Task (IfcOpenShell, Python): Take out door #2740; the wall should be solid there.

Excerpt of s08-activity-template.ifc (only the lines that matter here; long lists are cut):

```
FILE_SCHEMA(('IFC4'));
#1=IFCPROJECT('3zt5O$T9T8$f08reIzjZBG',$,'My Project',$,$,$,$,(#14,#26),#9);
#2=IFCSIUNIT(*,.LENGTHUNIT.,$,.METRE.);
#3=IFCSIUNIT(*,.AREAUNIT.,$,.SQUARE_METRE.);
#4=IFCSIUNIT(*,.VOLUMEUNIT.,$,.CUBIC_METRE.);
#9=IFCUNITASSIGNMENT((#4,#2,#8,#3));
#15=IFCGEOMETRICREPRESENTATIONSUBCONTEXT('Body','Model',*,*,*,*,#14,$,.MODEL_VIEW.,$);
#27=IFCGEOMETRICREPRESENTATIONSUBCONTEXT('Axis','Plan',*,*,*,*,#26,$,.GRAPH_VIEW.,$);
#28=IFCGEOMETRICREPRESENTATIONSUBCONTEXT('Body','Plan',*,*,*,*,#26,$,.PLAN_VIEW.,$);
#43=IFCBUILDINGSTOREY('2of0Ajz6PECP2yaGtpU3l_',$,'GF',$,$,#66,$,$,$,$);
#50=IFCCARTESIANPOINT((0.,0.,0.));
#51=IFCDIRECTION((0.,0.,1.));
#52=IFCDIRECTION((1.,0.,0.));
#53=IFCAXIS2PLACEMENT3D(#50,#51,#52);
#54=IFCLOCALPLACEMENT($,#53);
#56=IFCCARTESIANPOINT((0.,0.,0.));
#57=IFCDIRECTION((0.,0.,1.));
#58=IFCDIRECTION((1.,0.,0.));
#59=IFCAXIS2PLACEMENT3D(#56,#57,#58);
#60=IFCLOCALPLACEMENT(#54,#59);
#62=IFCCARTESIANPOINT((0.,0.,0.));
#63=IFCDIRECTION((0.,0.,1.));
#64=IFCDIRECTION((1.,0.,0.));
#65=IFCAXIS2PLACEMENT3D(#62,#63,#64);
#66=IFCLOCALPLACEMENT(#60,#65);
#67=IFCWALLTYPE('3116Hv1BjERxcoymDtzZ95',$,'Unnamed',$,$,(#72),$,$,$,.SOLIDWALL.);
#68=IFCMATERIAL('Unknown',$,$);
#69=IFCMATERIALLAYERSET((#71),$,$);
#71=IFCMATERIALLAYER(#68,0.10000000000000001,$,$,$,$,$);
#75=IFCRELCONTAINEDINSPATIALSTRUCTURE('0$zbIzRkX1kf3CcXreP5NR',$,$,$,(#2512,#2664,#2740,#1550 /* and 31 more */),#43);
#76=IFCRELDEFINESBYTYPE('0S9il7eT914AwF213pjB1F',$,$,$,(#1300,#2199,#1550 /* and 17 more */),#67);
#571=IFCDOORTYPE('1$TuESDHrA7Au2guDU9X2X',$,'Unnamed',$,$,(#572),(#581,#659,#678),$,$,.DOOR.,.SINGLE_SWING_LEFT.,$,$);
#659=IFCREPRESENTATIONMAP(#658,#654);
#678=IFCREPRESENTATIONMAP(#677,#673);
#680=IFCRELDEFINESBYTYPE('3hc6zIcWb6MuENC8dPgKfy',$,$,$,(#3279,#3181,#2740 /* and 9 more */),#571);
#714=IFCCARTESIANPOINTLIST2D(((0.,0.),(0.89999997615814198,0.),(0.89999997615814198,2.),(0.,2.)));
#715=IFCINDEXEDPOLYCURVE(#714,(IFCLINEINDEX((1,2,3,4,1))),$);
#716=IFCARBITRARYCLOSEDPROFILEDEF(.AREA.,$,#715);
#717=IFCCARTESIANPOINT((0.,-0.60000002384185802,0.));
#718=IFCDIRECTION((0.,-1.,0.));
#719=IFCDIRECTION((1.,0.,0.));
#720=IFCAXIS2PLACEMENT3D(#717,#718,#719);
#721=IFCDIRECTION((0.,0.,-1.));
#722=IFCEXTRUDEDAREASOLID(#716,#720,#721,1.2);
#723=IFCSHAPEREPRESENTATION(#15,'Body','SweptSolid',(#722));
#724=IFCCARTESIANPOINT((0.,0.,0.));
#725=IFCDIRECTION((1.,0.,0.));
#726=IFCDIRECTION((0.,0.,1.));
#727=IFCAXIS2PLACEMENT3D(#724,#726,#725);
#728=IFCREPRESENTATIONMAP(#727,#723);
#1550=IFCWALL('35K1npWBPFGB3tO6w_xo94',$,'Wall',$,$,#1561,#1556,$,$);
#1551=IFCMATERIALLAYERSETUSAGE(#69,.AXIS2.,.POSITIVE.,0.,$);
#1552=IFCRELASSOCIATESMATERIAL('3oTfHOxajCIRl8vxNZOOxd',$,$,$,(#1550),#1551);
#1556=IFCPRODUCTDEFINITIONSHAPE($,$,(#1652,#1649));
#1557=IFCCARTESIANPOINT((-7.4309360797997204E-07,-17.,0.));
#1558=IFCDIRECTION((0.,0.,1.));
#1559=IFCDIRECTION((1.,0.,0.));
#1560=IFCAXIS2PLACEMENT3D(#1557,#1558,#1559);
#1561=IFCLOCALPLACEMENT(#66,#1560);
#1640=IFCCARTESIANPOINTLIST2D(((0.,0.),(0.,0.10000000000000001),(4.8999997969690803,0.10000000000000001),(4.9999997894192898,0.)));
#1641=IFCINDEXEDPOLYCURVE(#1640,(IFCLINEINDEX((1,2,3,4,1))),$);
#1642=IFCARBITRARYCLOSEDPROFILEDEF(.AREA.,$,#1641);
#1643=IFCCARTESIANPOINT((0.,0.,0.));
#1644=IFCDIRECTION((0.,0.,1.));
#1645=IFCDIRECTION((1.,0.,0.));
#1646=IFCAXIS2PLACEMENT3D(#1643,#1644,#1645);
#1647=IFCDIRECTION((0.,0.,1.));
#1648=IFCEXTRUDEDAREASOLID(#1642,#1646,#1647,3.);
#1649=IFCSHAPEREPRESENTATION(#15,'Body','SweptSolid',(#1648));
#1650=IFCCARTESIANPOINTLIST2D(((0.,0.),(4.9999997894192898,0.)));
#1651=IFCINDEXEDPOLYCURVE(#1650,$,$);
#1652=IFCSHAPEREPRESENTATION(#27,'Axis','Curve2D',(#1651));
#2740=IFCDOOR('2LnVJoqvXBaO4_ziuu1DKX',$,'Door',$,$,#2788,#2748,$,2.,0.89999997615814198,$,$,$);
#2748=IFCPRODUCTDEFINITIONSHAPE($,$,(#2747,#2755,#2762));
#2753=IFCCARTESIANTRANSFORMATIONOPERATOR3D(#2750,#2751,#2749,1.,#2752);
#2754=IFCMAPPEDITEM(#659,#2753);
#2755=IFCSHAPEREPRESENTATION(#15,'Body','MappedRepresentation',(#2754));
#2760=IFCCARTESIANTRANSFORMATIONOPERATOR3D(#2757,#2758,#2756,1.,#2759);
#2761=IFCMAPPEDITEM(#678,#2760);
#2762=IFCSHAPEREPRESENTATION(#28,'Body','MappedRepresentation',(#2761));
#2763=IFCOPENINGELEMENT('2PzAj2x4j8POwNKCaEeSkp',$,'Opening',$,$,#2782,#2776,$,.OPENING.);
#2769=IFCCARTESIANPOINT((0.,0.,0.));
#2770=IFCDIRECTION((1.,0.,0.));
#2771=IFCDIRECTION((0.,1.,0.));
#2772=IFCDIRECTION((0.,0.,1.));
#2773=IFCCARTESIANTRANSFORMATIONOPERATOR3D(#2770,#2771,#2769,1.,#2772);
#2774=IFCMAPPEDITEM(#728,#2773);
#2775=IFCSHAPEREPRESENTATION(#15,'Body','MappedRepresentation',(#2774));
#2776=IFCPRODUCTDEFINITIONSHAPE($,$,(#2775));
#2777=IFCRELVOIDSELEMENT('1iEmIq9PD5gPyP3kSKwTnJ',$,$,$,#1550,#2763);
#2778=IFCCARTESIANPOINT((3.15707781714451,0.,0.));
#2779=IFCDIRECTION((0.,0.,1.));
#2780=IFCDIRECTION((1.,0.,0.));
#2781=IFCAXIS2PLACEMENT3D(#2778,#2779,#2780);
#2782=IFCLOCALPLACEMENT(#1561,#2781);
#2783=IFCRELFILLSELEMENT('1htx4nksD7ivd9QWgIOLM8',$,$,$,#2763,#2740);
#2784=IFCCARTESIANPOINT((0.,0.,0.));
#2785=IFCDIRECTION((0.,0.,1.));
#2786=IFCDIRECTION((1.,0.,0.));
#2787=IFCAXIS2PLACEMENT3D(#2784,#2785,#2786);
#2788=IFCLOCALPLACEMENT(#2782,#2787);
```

```python
import ifcopenshell
import ifcopenshell.api.feature
import ifcopenshell.api.root
import ifcopenshell.geom
import ifcopenshell.util.shape

model = ifcopenshell.open("s08-activity-template.ifc")
settings = ifcopenshell.geom.settings()


def volume(element):
    """Net volume in cubic metres, openings subtracted."""
    shape = ifcopenshell.geom.create_shape(settings, element)
    return ifcopenshell.util.shape.get_volume(shape.geometry)


door = model.by_guid("2LnVJoqvXBaO4_ziuu1DKX")
opening = door.FillsVoids[0].RelatingOpeningElement
wall = opening.VoidsElements[0].RelatingBuildingElement
before = volume(wall)

ifcopenshell.api.root.remove_product(model, product=door)
ifcopenshell.api.feature.remove_feature(model, feature=opening)

after = volume(wall)

print(f"wall volume {before:.3f} -> {after:.3f} m3")

model.write("s08-activity-template_rev.ifc")
```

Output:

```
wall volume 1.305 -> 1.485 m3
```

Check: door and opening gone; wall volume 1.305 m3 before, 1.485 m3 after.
